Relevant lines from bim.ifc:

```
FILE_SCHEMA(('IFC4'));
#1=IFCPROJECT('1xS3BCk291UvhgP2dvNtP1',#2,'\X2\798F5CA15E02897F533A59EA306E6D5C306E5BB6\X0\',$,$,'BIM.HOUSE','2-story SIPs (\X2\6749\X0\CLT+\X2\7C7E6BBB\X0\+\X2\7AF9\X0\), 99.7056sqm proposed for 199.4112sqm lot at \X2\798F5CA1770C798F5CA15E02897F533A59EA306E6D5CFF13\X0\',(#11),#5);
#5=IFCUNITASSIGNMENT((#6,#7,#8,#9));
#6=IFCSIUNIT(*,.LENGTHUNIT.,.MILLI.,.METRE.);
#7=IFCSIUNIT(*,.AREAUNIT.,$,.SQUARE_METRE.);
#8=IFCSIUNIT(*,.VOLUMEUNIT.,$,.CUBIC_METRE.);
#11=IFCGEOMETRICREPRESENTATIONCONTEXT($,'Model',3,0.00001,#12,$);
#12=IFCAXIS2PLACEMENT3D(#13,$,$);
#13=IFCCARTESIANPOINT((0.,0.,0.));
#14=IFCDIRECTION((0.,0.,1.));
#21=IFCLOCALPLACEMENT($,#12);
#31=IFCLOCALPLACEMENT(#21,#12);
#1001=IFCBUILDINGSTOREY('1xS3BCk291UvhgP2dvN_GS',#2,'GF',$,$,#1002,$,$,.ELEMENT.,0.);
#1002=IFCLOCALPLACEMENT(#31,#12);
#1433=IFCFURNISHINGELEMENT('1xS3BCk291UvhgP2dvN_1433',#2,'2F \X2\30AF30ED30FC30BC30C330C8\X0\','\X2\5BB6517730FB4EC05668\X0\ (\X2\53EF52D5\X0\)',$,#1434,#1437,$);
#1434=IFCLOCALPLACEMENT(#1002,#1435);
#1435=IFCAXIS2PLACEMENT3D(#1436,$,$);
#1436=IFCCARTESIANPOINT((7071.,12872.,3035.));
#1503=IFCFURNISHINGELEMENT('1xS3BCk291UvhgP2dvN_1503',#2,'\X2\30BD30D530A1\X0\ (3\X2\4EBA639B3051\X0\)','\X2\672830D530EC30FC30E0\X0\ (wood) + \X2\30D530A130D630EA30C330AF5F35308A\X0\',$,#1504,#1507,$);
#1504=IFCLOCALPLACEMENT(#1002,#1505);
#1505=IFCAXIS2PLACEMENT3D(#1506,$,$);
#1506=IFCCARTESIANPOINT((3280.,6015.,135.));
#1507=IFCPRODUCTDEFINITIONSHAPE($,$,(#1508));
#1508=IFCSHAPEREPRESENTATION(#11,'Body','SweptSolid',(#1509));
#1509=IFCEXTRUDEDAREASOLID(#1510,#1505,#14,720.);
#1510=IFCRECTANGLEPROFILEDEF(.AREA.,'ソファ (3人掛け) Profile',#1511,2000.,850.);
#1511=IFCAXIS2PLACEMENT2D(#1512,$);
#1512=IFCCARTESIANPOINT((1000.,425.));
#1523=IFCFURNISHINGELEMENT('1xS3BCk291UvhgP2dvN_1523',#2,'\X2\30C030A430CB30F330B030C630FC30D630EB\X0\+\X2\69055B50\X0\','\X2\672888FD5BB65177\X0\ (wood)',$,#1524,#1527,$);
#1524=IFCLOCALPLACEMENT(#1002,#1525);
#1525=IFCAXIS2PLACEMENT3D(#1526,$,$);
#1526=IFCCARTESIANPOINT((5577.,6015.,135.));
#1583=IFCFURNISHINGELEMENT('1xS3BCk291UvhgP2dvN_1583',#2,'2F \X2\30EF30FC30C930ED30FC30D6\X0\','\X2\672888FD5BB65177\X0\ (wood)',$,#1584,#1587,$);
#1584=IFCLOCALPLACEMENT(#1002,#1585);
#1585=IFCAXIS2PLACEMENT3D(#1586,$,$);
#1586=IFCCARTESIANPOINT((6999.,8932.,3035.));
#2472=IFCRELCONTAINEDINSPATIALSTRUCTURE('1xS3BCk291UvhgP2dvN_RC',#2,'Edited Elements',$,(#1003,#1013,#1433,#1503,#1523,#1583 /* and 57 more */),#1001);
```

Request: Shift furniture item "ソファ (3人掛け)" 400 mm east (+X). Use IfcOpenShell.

```python
import ifcopenshell
import ifcopenshell.api.geometry
import ifcopenshell.util.placement
import ifcopenshell.util.unit

model = ifcopenshell.open("bim.ifc")
unit_scale = ifcopenshell.util.unit.calculate_unit_scale(model)

item = model.by_guid("1xS3BCk291UvhgP2dvN_1503")
matrix = ifcopenshell.util.placement.get_local_placement(item.ObjectPlacement)
matrix[0, 3] += 0.4 / unit_scale
ifcopenshell.api.geometry.edit_object_placement(model, product=item, matrix=matrix, is_si=False)

print(ifcopenshell.util.placement.get_local_placement(item.ObjectPlacement).round(3) + 0.0)

model.write("bim_updated.ifc")
```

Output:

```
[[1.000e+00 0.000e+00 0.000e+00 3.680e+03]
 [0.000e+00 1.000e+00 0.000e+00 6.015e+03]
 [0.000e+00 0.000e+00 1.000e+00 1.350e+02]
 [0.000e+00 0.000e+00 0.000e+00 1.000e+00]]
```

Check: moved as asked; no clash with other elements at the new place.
